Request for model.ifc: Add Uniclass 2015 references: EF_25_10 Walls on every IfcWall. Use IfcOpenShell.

First a look at what the model holds.

```python
import ifcopenshell

model = ifcopenshell.open("model.ifc")
print(model.schema)
print("classifications:", [c.Name for c in model.by_type("IfcClassification")])
for ifc_class in ("IfcDoor", "IfcRoof", "IfcStair", "IfcWall", "IfcWindow"):
    print(ifc_class, len(model.by_type(ifc_class)))
```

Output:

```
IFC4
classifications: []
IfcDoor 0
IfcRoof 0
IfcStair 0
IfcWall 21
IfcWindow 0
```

```python
import ifcopenshell
import ifcopenshell.api.classification

model = ifcopenshell.open("model.ifc")

system = ifcopenshell.api.classification.add_classification(model, classification="Uniclass 2015")

codes = {
    "IfcWall": ("EF_25_10", "Walls"),
}
for ifc_class, (code, name) in codes.items():
    products = model.by_type(ifc_class)
    ifcopenshell.api.classification.add_reference(
        model, products=products, classification=system, identification=code, name=name
    )
    print(code, len(products))

model.write("model_edited.ifc")
```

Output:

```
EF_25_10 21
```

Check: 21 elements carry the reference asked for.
